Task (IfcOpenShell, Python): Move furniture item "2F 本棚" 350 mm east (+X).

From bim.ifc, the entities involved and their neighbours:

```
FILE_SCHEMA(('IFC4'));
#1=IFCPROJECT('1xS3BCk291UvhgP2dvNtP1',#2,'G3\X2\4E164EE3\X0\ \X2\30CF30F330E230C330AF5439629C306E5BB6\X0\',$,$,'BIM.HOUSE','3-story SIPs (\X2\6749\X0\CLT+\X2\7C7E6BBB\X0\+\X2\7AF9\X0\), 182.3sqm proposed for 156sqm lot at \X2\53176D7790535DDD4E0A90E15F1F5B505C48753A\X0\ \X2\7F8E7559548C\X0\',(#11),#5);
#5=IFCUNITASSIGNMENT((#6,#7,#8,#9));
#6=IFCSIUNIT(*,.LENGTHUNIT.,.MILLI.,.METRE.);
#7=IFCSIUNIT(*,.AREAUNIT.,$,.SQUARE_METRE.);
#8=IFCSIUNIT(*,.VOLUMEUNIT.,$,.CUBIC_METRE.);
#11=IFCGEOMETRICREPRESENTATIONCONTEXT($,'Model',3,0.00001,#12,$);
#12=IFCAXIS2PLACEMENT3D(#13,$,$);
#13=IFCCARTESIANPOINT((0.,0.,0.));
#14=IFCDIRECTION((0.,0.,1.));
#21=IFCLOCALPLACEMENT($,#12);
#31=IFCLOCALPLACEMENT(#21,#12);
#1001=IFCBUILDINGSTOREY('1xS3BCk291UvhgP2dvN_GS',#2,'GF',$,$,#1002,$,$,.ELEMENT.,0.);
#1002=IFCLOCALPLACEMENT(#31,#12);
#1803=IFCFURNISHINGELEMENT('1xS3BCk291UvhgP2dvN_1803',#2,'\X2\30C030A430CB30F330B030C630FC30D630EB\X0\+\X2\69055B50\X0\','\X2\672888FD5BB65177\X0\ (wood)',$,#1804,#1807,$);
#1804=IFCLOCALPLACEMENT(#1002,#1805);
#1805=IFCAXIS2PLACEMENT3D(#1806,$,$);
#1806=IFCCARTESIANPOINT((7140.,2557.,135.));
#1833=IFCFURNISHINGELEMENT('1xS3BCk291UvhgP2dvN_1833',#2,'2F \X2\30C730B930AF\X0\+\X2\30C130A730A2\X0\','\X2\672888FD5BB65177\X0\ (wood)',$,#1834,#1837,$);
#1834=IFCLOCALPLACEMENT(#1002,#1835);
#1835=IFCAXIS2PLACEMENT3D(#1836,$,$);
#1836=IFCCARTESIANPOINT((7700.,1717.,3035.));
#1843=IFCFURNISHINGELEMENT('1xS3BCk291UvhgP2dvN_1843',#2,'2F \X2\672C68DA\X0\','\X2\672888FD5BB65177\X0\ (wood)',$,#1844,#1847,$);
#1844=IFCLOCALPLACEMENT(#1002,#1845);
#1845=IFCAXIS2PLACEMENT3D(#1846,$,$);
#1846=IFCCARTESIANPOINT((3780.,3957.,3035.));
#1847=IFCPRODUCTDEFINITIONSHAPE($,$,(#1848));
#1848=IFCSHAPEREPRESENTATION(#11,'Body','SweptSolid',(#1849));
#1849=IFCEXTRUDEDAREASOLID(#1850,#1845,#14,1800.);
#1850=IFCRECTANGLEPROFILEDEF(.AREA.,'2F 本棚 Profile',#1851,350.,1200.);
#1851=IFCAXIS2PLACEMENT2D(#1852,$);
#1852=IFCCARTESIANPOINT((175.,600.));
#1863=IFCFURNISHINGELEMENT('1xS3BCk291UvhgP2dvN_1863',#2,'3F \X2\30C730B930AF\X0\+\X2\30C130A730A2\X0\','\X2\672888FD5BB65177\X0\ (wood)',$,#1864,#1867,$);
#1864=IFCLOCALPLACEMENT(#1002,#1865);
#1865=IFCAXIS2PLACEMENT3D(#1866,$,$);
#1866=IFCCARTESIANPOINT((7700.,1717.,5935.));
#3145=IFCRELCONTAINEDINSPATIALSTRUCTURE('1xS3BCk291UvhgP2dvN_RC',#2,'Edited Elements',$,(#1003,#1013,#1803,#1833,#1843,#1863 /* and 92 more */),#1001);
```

```python
import ifcopenshell
import ifcopenshell.api.geometry
import ifcopenshell.util.placement

model = ifcopenshell.open("bim.ifc")

item = model.by_guid("1xS3BCk291UvhgP2dvN_1843")
matrix = ifcopenshell.util.placement.get_local_placement(item.ObjectPlacement)
matrix[0, 3] += 350.0
ifcopenshell.api.geometry.edit_object_placement(model, product=item, matrix=matrix, is_si=False)

print(ifcopenshell.util.placement.get_local_placement(item.ObjectPlacement).round(3) + 0.0)

model.write("bim_updated.ifc")
```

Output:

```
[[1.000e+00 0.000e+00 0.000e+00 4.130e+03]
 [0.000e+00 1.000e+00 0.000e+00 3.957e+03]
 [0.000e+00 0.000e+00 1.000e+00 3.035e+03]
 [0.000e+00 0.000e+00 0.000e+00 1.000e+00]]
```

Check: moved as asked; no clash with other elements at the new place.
